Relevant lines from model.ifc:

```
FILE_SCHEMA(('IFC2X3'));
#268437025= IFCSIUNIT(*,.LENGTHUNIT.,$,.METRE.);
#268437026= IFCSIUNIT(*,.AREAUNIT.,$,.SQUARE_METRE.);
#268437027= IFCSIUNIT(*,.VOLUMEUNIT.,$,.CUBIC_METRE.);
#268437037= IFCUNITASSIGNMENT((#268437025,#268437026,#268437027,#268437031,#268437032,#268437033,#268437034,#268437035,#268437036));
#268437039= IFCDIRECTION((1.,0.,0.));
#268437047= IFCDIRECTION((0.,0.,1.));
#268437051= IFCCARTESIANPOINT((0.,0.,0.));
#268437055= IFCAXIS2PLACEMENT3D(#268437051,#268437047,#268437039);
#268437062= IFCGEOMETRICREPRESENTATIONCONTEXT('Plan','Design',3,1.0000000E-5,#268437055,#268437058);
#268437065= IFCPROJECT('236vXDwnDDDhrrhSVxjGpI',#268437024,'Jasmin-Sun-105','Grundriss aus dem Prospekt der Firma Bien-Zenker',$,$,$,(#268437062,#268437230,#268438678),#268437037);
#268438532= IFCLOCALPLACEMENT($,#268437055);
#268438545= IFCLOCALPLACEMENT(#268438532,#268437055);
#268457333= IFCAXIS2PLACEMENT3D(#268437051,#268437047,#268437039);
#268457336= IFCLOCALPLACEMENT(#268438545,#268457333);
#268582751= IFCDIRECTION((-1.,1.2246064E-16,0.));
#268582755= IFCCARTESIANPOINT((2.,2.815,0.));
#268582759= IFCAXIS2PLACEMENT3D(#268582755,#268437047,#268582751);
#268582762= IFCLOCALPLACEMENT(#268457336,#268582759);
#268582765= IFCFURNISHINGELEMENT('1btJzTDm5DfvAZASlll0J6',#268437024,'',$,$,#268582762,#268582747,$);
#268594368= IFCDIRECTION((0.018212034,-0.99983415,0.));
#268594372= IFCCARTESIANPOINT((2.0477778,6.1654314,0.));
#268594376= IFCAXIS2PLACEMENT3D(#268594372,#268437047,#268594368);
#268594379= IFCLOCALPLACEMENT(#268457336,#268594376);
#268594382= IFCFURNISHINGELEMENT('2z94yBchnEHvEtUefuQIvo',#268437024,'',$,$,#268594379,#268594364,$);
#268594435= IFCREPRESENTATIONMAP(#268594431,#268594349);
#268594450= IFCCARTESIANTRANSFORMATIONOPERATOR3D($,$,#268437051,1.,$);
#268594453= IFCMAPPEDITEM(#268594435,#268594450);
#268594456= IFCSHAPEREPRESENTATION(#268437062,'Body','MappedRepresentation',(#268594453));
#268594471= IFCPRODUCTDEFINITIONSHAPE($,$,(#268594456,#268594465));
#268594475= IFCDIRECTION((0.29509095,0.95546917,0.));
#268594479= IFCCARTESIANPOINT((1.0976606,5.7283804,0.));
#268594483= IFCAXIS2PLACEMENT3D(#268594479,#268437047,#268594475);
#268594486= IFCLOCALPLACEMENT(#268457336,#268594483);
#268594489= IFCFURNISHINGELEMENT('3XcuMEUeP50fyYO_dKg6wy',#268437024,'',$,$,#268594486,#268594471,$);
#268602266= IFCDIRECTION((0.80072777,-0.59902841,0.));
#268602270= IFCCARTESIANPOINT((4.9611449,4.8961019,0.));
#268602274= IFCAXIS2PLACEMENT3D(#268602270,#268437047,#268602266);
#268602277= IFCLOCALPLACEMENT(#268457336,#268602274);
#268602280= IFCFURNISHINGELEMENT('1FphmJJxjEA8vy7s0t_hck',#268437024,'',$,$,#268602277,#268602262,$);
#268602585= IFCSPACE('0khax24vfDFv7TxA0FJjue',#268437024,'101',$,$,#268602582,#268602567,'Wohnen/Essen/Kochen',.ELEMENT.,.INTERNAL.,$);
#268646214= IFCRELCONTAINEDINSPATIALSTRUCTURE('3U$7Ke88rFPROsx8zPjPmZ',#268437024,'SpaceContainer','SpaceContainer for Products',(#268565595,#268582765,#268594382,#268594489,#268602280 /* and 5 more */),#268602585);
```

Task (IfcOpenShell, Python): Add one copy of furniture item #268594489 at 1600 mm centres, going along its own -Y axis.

```python
import ifcopenshell
import ifcopenshell.api.geometry
import ifcopenshell.api.root
import ifcopenshell.util.element
import ifcopenshell.util.placement
import ifcopenshell.util.unit

model = ifcopenshell.open("model.ifc")
unit_scale = ifcopenshell.util.unit.calculate_unit_scale(model)


def reuse_history(source, copy):
    """copy_class also copies each property set's owner history, people and application; keep the originals."""
    for rel in copy.IsDefinedBy:
        if rel.is_a("IfcRelDefinesByProperties") and (history := rel.RelatingPropertyDefinition.OwnerHistory):
            rel.RelatingPropertyDefinition.OwnerHistory = source.OwnerHistory
            ifcopenshell.util.element.remove_deep2(model, history)


source = model.by_id(268594489)
base = ifcopenshell.util.placement.get_local_placement(source.ObjectPlacement)
step = -base[:3, 1] * 1.6 / unit_scale

for i in range(1, 2):
    copy = ifcopenshell.api.root.copy_class(model, product=source)
    copy.Representation = ifcopenshell.util.element.copy_deep(
        model, source.Representation, exclude=["IfcGeometricRepresentationContext", "IfcRepresentationMap"]
    )
    reuse_history(source, copy)
    matrix = base.copy()
    matrix[:3, 3] += i * step
    print("added at", matrix[:3, 3].round(3) + 0.0)
    ifcopenshell.api.geometry.edit_object_placement(model, product=copy, matrix=matrix, is_si=False)

model.write("model_updated.ifc")
```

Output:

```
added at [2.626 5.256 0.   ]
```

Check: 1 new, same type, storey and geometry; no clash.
